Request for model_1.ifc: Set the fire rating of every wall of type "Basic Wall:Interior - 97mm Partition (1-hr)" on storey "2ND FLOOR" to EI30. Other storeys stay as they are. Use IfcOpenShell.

First a look at what the model holds.

```python
import ifcopenshell
import ifcopenshell.util.element

model = ifcopenshell.open("model_1.ifc")
print(model.schema)
storey = next(s for s in model.by_type("IfcBuildingStorey") if s.Name == "2ND FLOOR")
walls = [e for e in ifcopenshell.util.element.get_decomposition(storey) if e.is_a("IfcWall")]
seen = {}
for e in walls:
    element_type = ifcopenshell.util.element.get_type(e)
    key = (element_type.Name if element_type != e and element_type else None, ifcopenshell.util.element.get_pset(e, "Pset_WallCommon", "FireRating"))
    seen[key] = seen.get(key, 0) + 1
for (name, value), count in sorted(seen.items(), key=str):
    print(count, "x", name, "|", value)
```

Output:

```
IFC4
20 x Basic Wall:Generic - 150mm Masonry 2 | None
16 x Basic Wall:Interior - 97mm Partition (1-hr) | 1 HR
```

```python
import ifcopenshell
import ifcopenshell.api.pset
import ifcopenshell.util.element

model = ifcopenshell.open("model_1.ifc")

storey = next(s for s in model.by_type("IfcBuildingStorey") if s.Name == "2ND FLOOR")
walls = [e for e in ifcopenshell.util.element.get_decomposition(storey) if e.is_a("IfcWall")]

count = 0
for e in walls:
    element_type = ifcopenshell.util.element.get_type(e)
    if element_type in (None, e) or element_type.Name != "Basic Wall:Interior - 97mm Partition (1-hr)":
        continue
    # add_pset returns the element's existing set when there is one.
    pset = ifcopenshell.api.pset.add_pset(model, product=e, name="Pset_WallCommon")
    ifcopenshell.api.pset.edit_pset(model, pset=pset, properties={"FireRating": "EI30"})
    count += 1

print(count, "walls updated")

model.write("model_1_edited.ifc")
```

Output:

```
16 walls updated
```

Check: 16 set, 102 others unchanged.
